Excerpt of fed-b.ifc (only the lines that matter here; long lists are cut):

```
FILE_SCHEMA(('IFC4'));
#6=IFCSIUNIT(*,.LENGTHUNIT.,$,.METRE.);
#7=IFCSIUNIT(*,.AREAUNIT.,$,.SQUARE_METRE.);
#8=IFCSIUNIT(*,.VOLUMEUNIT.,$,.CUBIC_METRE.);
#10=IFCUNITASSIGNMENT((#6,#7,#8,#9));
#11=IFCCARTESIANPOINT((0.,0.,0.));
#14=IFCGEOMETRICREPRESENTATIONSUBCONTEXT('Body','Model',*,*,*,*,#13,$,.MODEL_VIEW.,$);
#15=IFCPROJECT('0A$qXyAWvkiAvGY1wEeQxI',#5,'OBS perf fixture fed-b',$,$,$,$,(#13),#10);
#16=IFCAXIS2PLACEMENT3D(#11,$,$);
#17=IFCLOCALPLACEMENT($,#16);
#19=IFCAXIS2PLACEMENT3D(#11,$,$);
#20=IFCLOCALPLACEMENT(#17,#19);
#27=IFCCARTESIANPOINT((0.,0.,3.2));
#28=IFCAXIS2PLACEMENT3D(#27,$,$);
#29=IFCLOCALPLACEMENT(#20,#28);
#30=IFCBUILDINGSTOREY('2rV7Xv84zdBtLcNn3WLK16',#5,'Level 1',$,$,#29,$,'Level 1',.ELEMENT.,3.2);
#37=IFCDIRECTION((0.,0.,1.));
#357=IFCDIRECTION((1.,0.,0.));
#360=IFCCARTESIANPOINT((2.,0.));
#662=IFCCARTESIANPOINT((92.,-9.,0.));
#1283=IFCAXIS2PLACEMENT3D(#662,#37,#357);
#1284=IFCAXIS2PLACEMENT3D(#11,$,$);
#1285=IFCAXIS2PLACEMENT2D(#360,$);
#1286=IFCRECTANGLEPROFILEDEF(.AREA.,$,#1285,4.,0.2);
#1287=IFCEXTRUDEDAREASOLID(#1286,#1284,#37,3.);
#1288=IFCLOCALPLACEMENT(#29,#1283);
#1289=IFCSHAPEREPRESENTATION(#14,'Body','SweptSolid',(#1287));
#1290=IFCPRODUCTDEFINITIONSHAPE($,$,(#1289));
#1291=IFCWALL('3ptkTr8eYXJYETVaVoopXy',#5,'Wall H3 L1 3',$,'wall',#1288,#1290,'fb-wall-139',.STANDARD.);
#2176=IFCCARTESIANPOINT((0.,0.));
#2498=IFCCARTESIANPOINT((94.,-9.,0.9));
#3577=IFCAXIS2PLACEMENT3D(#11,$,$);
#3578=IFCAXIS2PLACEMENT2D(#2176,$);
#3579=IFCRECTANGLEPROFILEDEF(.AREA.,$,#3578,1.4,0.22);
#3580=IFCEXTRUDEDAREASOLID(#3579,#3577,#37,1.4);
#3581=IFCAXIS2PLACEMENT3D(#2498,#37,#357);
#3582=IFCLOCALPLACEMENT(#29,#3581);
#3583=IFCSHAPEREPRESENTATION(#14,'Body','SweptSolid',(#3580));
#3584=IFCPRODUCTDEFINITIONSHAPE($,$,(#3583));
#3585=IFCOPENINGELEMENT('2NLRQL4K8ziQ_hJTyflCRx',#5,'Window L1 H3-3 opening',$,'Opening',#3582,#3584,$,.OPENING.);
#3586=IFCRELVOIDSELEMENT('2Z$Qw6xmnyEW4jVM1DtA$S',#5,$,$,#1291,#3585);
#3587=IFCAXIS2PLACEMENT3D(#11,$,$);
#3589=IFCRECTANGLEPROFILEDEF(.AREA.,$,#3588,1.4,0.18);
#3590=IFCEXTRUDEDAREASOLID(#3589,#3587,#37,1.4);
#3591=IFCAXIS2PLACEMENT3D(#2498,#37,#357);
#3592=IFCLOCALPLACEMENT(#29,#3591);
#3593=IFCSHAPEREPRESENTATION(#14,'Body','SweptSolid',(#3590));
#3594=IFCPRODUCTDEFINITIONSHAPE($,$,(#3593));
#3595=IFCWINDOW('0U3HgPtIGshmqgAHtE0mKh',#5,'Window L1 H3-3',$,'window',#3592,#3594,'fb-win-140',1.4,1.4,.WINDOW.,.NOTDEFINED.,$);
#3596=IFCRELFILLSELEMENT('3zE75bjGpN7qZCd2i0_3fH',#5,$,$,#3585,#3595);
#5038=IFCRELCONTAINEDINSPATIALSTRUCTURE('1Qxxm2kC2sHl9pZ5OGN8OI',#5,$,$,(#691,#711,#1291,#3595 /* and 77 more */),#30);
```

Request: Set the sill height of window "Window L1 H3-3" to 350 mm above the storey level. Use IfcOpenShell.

```python
import numpy as np
import ifcopenshell
import ifcopenshell.api.geometry
import ifcopenshell.geom
import ifcopenshell.util.element
import ifcopenshell.util.placement
import ifcopenshell.util.shape
import ifcopenshell.util.unit

model = ifcopenshell.open("fed-b.ifc")
unit_scale = ifcopenshell.util.unit.calculate_unit_scale(model)

window = model.by_id(3595)
opening = window.FillsVoids[0].RelatingOpeningElement
storey = ifcopenshell.util.element.get_container(window, ifc_class="IfcBuildingStorey")
level = ifcopenshell.util.placement.get_local_placement(storey.ObjectPlacement)[2, 3]

# The opening's origin need not be at the sill, so measure its lowest point.
shape = ifcopenshell.geom.create_shape(ifcopenshell.geom.settings(), opening)
bottom = ifcopenshell.util.shape.get_shape_bottom_elevation(shape, shape.geometry) / unit_scale
dz = level + 0.35 - bottom

shift = np.array([0.0, 0.0, dz])
# The window is not placed relative to its opening, so move both.
for product in (opening, window):
    matrix = ifcopenshell.util.placement.get_local_placement(product.ObjectPlacement)
    matrix[:3, 3] += shift
    ifcopenshell.api.geometry.edit_object_placement(model, product=product, matrix=matrix, is_si=False)

print(f"moved by {dz * unit_scale:+.3f} m")

model.write("fed-b_updated.ifc")
```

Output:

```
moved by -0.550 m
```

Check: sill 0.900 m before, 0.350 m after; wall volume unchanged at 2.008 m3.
